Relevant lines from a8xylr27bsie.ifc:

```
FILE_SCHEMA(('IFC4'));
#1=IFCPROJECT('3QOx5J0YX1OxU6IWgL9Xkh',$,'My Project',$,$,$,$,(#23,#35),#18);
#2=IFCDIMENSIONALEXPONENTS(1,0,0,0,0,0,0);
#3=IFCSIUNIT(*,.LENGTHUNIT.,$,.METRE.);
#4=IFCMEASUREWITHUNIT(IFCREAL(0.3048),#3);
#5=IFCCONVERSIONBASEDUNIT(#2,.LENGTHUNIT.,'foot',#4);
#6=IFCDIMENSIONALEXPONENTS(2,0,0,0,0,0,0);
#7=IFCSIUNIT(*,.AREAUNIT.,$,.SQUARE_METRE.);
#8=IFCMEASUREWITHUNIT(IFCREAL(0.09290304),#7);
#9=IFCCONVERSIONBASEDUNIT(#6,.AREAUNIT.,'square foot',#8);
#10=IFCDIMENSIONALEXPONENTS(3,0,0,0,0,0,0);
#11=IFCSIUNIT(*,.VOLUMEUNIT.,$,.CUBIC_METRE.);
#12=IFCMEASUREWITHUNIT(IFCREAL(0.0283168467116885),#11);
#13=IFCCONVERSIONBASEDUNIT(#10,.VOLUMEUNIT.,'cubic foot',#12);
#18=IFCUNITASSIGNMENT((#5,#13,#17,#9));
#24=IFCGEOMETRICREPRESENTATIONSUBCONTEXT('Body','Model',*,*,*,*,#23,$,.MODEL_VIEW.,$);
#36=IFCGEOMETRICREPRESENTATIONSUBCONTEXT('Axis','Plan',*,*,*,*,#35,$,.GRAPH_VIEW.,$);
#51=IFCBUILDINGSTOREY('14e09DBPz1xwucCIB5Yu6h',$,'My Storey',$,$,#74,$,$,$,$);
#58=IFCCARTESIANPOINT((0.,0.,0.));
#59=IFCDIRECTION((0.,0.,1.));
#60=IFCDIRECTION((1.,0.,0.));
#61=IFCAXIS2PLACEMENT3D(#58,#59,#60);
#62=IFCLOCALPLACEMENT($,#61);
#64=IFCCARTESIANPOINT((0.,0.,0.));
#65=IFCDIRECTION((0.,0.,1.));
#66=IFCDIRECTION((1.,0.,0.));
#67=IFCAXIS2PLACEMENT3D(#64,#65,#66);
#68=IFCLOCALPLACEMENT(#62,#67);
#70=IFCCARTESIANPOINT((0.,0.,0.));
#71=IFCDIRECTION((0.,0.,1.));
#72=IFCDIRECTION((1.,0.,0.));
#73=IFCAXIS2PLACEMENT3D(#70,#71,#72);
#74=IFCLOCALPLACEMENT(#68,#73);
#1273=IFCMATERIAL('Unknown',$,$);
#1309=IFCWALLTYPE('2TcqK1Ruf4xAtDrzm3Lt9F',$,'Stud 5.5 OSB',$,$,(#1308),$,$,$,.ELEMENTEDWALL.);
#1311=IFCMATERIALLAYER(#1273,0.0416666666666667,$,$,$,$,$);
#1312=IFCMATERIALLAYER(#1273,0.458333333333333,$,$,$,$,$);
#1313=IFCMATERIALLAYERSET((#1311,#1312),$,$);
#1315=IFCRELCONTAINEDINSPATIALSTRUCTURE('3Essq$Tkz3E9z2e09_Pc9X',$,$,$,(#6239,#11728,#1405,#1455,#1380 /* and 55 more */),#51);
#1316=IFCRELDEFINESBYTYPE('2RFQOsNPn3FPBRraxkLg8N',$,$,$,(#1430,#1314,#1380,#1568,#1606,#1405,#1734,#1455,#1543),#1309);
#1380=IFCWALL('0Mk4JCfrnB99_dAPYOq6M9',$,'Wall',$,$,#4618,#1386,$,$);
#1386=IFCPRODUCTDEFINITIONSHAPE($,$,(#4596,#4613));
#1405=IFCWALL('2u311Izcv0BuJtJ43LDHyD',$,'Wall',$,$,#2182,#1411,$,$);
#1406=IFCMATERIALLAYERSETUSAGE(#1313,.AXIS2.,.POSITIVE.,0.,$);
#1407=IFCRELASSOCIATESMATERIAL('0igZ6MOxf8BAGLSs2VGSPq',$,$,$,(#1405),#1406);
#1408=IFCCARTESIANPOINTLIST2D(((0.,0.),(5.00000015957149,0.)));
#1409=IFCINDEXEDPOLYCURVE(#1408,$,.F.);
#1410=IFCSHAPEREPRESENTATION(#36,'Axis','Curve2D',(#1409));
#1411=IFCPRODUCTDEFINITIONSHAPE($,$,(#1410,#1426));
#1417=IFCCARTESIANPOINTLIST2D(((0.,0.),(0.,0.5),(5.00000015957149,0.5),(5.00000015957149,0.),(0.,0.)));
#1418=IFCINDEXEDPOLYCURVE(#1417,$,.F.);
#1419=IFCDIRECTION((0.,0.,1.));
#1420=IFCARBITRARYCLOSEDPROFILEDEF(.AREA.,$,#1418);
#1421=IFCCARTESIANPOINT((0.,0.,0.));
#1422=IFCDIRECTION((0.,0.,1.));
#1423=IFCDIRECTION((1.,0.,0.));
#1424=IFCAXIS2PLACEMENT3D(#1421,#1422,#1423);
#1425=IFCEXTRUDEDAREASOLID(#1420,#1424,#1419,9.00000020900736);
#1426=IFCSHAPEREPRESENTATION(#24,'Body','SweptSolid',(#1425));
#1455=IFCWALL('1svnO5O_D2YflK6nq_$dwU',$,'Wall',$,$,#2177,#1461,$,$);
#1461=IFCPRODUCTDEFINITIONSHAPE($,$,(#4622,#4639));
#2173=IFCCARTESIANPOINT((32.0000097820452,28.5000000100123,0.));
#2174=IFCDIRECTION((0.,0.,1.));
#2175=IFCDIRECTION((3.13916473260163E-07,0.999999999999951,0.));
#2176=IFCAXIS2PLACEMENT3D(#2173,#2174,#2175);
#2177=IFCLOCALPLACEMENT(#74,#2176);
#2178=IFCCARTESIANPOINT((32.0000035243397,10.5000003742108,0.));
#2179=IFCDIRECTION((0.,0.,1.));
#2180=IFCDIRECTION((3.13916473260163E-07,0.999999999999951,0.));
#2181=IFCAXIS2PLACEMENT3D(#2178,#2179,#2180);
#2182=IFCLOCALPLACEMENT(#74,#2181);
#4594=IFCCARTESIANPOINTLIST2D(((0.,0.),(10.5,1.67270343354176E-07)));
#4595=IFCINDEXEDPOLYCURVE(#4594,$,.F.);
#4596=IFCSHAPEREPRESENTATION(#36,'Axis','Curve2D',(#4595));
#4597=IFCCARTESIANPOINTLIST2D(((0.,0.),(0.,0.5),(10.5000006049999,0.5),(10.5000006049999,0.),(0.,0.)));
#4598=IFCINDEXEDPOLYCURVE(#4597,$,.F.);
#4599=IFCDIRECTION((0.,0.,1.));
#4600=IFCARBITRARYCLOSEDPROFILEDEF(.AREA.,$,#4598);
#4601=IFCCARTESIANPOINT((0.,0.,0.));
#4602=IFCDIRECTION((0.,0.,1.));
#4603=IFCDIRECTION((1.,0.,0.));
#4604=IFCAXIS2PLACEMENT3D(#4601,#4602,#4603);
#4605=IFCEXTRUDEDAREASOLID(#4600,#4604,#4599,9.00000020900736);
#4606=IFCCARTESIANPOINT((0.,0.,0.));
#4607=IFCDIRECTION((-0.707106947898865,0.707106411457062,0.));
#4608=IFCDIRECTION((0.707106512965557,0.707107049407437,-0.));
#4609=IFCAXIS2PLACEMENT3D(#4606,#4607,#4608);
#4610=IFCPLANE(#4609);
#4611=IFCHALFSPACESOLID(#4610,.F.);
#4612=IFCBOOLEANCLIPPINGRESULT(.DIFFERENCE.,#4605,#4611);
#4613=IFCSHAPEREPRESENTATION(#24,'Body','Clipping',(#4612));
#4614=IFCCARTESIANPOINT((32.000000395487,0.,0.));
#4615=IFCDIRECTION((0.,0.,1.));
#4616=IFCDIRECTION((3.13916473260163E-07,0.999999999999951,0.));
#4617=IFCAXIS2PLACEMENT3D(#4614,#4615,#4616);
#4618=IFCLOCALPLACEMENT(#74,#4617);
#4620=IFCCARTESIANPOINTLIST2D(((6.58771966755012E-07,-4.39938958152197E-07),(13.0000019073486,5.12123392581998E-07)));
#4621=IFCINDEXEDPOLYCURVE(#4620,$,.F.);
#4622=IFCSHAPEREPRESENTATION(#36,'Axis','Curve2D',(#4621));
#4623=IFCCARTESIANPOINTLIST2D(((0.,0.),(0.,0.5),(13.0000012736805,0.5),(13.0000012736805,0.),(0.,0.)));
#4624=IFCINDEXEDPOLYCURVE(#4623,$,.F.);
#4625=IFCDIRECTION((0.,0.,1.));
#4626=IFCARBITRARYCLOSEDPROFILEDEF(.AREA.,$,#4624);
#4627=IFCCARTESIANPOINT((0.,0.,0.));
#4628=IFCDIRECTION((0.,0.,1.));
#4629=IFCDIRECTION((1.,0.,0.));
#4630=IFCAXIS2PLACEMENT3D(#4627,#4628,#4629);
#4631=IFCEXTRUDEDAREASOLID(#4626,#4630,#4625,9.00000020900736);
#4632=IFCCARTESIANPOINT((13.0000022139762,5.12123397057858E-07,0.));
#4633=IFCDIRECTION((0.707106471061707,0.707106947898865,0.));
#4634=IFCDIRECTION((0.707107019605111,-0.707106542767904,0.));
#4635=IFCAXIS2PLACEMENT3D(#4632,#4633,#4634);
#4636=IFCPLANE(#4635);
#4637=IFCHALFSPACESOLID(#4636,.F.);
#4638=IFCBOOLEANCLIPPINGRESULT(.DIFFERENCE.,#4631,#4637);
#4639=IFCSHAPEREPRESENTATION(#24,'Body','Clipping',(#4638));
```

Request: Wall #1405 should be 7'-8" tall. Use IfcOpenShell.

```python
import ifcopenshell
import ifcopenshell.geom
import ifcopenshell.util.representation
import ifcopenshell.util.shape
import ifcopenshell.util.unit

model = ifcopenshell.open("a8xylr27bsie.ifc")
unit_scale = ifcopenshell.util.unit.calculate_unit_scale(model)
settings = ifcopenshell.geom.settings()


def volume(element):
    """Net volume in cubic metres, openings subtracted."""
    shape = ifcopenshell.geom.create_shape(settings, element)
    return ifcopenshell.util.shape.get_volume(shape.geometry)


wall = model.by_guid("2u311Izcv0BuJtJ43LDHyD")
before = volume(wall)

body = ifcopenshell.util.representation.get_representation(wall, "Model", "Body")
solid = body.Items[0]
old_height = solid.Depth
solid.Depth = 92 * 0.0254 / unit_scale
after = volume(wall)

print(f"height {old_height:g} -> {solid.Depth:g}, volume {before:.3f} -> {after:.3f} m3")

model.write("a8xylr27bsie_edited.ifc")
```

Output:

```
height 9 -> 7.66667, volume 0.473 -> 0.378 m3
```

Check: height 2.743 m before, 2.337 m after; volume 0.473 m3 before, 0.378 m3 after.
